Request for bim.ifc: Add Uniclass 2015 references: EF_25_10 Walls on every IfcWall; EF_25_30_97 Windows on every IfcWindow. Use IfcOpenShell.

First a look at what the model holds.

```python
import ifcopenshell

model = ifcopenshell.open("bim.ifc")
print(model.schema)
print("classifications:", [c.Name for c in model.by_type("IfcClassification")])
for ifc_class in ("IfcDoor", "IfcRoof", "IfcStair", "IfcWall", "IfcWindow"):
    print(ifc_class, len(model.by_type(ifc_class)))
```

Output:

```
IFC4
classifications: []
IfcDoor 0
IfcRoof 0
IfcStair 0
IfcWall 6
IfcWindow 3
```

```python
import ifcopenshell
import ifcopenshell.api.classification

model = ifcopenshell.open("bim.ifc")

system = ifcopenshell.api.classification.add_classification(model, classification="Uniclass 2015")

codes = {
    "IfcWall": ("EF_25_10", "Walls"),
    "IfcWindow": ("EF_25_30_97", "Windows"),
}
for ifc_class, (code, name) in codes.items():
    products = model.by_type(ifc_class)
    ifcopenshell.api.classification.add_reference(
        model, products=products, classification=system, identification=code, name=name
    )
    print(code, len(products))

model.write("bim_v2.ifc")
```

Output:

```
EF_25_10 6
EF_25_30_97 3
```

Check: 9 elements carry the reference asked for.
